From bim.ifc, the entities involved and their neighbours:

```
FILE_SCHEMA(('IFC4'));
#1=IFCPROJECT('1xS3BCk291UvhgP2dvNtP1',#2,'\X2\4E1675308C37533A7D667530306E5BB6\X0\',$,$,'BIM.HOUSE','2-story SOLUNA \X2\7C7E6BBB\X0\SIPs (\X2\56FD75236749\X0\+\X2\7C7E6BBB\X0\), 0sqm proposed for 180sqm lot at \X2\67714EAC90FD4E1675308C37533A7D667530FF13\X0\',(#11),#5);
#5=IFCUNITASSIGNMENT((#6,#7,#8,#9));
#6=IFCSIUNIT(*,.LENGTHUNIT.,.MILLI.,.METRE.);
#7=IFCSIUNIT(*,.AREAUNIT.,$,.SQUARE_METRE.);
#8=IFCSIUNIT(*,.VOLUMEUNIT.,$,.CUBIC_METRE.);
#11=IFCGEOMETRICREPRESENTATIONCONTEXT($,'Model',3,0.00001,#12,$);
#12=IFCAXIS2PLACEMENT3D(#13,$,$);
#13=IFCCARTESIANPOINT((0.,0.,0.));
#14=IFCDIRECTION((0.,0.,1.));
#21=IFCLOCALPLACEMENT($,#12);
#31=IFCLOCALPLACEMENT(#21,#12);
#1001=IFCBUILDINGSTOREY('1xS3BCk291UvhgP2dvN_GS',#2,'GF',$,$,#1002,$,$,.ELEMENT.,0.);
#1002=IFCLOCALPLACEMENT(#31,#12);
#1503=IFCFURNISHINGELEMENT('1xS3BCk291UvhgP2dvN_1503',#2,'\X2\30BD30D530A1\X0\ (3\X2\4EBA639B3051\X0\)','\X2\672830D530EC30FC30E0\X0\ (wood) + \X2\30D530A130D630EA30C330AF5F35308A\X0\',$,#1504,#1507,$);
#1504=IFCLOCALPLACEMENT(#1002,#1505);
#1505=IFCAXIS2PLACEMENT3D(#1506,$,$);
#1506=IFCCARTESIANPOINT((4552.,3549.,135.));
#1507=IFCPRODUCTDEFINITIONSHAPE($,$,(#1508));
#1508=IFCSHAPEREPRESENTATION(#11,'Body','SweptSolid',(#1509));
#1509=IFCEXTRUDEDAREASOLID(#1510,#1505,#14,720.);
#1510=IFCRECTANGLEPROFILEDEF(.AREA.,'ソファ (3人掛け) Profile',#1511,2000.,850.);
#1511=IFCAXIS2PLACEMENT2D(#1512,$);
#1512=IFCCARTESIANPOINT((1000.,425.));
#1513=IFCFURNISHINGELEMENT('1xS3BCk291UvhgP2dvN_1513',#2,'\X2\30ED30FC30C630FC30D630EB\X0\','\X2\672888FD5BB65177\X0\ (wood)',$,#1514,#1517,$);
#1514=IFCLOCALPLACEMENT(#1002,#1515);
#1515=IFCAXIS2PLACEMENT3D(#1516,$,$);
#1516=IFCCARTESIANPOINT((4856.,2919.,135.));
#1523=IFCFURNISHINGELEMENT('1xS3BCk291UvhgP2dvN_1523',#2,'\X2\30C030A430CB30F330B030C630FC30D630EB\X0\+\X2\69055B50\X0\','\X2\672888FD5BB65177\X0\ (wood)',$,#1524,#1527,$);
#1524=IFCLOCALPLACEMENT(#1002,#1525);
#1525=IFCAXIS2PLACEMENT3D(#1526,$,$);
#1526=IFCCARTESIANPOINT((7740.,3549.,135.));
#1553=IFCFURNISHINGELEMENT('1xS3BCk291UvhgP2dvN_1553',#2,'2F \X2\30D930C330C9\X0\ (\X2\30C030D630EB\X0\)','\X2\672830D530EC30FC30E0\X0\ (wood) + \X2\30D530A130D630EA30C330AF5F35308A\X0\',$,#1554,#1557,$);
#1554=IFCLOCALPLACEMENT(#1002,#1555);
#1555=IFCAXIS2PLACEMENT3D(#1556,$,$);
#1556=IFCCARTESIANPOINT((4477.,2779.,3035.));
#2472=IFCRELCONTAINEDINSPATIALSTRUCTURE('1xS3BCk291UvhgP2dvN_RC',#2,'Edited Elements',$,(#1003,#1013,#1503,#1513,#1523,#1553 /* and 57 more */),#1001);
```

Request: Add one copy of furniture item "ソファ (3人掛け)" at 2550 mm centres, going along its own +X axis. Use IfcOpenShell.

```python
import ifcopenshell
import ifcopenshell.api.geometry
import ifcopenshell.api.root
import ifcopenshell.util.element
import ifcopenshell.util.placement

model = ifcopenshell.open("bim.ifc")


def reuse_history(source, copy):
    """copy_class also copies each property set's owner history, people and application; keep the originals."""
    for rel in copy.IsDefinedBy:
        if rel.is_a("IfcRelDefinesByProperties") and (history := rel.RelatingPropertyDefinition.OwnerHistory):
            rel.RelatingPropertyDefinition.OwnerHistory = source.OwnerHistory
            ifcopenshell.util.element.remove_deep2(model, history)


source = model.by_guid("1xS3BCk291UvhgP2dvN_1503")
base = ifcopenshell.util.placement.get_local_placement(source.ObjectPlacement)
step = base[:3, 0] * 2550.0

for i in range(1, 2):
    copy = ifcopenshell.api.root.copy_class(model, product=source)
    copy.Representation = ifcopenshell.util.element.copy_deep(
        model, source.Representation, exclude=["IfcGeometricRepresentationContext", "IfcRepresentationMap"]
    )
    reuse_history(source, copy)
    matrix = base.copy()
    matrix[:3, 3] += i * step
    print("added at", matrix[:3, 3].round(3) + 0.0)
    ifcopenshell.api.geometry.edit_object_placement(model, product=copy, matrix=matrix, is_si=False)

model.write("bim-out.ifc")
```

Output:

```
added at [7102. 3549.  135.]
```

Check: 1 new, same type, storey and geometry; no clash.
